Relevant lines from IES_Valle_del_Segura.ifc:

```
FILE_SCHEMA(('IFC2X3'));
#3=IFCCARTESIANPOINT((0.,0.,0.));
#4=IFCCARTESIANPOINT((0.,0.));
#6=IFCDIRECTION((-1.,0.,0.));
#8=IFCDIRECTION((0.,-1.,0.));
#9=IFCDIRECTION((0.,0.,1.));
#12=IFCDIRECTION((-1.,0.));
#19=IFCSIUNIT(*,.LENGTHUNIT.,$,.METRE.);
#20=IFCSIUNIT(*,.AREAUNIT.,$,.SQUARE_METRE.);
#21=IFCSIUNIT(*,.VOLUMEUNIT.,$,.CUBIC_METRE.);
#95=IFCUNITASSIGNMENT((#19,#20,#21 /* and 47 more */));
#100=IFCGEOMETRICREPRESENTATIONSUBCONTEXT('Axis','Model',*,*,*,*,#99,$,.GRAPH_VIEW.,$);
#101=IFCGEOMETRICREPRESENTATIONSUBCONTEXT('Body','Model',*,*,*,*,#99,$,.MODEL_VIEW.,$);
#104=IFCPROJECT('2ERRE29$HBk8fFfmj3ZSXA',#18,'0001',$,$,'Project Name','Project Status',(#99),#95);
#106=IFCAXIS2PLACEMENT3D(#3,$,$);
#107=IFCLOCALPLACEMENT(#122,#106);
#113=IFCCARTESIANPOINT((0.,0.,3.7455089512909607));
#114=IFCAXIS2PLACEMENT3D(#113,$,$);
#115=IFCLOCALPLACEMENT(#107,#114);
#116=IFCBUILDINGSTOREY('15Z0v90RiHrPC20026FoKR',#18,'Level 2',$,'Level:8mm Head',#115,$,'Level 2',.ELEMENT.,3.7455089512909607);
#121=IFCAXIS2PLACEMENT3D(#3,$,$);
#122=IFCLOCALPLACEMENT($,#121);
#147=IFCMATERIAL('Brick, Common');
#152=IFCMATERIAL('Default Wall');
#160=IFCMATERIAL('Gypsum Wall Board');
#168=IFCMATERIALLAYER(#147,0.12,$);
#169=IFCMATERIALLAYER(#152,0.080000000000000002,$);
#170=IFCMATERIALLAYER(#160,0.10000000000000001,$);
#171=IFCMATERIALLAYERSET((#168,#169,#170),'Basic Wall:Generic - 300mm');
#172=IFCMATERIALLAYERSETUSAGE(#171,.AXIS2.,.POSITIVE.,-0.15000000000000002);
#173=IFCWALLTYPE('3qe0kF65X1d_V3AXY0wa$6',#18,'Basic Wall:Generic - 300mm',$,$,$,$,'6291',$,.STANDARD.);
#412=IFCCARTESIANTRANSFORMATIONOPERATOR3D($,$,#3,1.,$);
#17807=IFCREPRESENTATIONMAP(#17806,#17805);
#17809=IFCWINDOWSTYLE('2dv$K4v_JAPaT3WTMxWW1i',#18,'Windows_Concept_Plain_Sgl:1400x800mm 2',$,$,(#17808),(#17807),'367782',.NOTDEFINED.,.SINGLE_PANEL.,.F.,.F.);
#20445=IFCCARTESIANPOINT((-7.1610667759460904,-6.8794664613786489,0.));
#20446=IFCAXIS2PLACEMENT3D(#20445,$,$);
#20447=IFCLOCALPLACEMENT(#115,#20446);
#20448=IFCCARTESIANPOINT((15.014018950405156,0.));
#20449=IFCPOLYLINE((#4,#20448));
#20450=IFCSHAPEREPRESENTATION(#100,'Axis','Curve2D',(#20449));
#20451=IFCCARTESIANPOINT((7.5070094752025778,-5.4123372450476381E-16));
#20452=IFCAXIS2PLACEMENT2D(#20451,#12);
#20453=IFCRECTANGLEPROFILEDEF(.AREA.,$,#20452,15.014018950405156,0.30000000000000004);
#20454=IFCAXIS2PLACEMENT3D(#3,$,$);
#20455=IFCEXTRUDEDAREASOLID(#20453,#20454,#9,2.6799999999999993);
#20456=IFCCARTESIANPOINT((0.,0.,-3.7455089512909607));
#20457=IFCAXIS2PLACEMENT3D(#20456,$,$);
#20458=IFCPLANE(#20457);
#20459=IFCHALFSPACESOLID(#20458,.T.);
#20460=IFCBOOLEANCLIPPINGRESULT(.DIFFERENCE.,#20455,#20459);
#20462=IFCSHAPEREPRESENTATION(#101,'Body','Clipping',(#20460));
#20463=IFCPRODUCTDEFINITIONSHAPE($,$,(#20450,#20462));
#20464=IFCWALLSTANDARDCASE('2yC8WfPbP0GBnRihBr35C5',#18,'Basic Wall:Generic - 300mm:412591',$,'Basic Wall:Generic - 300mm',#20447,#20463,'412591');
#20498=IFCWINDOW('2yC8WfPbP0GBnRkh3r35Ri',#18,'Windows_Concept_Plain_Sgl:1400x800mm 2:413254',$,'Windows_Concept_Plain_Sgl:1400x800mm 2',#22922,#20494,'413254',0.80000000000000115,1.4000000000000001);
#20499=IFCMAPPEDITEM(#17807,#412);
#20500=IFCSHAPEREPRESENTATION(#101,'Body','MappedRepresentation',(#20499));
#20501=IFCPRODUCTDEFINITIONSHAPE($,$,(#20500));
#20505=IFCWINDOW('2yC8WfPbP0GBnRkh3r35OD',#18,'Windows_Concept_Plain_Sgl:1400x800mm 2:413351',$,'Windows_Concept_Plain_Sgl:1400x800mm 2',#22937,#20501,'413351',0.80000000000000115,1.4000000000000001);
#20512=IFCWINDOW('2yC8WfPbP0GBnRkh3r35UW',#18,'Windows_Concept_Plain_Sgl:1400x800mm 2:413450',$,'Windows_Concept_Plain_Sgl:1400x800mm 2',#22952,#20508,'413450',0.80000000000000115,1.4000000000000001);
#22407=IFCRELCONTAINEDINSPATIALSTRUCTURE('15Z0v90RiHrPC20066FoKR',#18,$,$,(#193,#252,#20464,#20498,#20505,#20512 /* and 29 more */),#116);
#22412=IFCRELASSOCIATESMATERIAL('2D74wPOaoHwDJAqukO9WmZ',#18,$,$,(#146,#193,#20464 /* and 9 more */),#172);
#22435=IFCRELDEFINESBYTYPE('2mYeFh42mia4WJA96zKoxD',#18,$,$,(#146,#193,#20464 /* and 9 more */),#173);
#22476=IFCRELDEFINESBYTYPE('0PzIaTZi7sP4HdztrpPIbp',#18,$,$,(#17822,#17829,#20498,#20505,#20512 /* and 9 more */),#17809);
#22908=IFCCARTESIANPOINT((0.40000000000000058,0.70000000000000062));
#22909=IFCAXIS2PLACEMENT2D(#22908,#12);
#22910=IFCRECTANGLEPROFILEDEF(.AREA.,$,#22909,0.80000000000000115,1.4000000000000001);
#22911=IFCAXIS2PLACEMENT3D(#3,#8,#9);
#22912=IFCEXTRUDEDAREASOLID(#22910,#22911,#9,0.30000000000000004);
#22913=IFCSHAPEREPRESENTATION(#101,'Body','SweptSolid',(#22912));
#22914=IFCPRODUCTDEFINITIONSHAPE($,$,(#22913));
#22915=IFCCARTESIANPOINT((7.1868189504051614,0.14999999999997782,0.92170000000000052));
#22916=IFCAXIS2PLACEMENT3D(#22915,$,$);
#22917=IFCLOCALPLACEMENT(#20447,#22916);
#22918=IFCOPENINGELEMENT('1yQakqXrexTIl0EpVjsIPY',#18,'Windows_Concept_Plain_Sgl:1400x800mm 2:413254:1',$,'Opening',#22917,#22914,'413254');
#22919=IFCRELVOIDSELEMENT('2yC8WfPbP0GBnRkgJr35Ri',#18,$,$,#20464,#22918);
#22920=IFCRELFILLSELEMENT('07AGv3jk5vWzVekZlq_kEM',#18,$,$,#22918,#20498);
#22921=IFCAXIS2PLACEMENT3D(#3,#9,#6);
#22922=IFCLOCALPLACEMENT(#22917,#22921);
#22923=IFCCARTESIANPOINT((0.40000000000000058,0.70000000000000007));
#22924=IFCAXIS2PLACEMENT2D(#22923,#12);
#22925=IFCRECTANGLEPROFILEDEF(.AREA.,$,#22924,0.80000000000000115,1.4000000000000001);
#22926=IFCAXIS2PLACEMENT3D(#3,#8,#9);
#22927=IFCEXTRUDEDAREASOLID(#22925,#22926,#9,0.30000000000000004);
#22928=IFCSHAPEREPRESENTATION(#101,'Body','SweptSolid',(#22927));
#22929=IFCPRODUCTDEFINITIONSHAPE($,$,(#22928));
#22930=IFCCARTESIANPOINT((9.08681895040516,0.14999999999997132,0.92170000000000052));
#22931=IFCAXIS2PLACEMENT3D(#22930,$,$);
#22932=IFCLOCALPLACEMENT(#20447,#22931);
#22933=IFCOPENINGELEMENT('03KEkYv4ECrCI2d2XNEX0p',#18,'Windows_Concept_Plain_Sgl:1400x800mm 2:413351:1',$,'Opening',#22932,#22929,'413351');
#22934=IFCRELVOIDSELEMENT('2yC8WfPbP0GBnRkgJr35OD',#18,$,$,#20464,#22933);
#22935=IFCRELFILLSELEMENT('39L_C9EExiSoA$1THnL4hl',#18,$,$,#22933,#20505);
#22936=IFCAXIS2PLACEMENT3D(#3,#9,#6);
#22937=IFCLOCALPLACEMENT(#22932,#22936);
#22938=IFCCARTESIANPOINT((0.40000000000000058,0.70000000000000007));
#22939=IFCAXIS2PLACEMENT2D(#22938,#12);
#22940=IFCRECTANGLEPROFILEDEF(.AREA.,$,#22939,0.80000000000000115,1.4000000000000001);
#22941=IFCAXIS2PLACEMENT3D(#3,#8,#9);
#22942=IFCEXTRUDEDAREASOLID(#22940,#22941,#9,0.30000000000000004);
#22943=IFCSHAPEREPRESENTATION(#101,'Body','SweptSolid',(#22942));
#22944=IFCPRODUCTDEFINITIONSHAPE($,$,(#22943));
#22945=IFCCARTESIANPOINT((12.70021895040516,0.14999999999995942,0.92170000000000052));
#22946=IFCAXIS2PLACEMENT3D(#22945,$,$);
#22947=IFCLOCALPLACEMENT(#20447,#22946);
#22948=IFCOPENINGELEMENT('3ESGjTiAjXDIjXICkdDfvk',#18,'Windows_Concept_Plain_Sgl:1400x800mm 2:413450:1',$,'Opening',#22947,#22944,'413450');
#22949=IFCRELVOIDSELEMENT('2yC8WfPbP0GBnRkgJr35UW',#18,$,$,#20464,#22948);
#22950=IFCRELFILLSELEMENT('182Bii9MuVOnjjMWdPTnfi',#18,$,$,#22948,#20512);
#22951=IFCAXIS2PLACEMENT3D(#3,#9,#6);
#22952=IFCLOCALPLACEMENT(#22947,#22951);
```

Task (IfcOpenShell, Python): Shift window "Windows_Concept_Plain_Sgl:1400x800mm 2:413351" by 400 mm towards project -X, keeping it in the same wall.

```python
import ifcopenshell
import ifcopenshell.api.geometry
import ifcopenshell.util.placement
import ifcopenshell.util.unit

model = ifcopenshell.open("IES_Valle_del_Segura.ifc")
unit_scale = ifcopenshell.util.unit.calculate_unit_scale(model)

window = model.by_id(20505)
opening = window.FillsVoids[0].RelatingOpeningElement
wall = opening.VoidsElements[0].RelatingBuildingElement

wall_matrix = ifcopenshell.util.placement.get_local_placement(wall.ObjectPlacement)
shift = wall_matrix[:3, 0] * -0.4 / unit_scale
before = ifcopenshell.util.placement.get_local_placement(window.ObjectPlacement)[:3, 3].copy()

# The window is placed relative to its opening, so it follows when the opening moves.
matrix = ifcopenshell.util.placement.get_local_placement(opening.ObjectPlacement)
matrix[:3, 3] += shift
ifcopenshell.api.geometry.edit_object_placement(
    model, product=opening, matrix=matrix, is_si=False, should_transform_children=True
)

after = ifcopenshell.util.placement.get_local_placement(window.ObjectPlacement)[:3, 3]
print("window moved by", (after - before).round(3) + 0.0)

model.write("IES_Valle_del_Segura_rev.ifc")
```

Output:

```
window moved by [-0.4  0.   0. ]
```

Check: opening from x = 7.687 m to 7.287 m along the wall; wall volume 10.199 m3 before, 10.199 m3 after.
